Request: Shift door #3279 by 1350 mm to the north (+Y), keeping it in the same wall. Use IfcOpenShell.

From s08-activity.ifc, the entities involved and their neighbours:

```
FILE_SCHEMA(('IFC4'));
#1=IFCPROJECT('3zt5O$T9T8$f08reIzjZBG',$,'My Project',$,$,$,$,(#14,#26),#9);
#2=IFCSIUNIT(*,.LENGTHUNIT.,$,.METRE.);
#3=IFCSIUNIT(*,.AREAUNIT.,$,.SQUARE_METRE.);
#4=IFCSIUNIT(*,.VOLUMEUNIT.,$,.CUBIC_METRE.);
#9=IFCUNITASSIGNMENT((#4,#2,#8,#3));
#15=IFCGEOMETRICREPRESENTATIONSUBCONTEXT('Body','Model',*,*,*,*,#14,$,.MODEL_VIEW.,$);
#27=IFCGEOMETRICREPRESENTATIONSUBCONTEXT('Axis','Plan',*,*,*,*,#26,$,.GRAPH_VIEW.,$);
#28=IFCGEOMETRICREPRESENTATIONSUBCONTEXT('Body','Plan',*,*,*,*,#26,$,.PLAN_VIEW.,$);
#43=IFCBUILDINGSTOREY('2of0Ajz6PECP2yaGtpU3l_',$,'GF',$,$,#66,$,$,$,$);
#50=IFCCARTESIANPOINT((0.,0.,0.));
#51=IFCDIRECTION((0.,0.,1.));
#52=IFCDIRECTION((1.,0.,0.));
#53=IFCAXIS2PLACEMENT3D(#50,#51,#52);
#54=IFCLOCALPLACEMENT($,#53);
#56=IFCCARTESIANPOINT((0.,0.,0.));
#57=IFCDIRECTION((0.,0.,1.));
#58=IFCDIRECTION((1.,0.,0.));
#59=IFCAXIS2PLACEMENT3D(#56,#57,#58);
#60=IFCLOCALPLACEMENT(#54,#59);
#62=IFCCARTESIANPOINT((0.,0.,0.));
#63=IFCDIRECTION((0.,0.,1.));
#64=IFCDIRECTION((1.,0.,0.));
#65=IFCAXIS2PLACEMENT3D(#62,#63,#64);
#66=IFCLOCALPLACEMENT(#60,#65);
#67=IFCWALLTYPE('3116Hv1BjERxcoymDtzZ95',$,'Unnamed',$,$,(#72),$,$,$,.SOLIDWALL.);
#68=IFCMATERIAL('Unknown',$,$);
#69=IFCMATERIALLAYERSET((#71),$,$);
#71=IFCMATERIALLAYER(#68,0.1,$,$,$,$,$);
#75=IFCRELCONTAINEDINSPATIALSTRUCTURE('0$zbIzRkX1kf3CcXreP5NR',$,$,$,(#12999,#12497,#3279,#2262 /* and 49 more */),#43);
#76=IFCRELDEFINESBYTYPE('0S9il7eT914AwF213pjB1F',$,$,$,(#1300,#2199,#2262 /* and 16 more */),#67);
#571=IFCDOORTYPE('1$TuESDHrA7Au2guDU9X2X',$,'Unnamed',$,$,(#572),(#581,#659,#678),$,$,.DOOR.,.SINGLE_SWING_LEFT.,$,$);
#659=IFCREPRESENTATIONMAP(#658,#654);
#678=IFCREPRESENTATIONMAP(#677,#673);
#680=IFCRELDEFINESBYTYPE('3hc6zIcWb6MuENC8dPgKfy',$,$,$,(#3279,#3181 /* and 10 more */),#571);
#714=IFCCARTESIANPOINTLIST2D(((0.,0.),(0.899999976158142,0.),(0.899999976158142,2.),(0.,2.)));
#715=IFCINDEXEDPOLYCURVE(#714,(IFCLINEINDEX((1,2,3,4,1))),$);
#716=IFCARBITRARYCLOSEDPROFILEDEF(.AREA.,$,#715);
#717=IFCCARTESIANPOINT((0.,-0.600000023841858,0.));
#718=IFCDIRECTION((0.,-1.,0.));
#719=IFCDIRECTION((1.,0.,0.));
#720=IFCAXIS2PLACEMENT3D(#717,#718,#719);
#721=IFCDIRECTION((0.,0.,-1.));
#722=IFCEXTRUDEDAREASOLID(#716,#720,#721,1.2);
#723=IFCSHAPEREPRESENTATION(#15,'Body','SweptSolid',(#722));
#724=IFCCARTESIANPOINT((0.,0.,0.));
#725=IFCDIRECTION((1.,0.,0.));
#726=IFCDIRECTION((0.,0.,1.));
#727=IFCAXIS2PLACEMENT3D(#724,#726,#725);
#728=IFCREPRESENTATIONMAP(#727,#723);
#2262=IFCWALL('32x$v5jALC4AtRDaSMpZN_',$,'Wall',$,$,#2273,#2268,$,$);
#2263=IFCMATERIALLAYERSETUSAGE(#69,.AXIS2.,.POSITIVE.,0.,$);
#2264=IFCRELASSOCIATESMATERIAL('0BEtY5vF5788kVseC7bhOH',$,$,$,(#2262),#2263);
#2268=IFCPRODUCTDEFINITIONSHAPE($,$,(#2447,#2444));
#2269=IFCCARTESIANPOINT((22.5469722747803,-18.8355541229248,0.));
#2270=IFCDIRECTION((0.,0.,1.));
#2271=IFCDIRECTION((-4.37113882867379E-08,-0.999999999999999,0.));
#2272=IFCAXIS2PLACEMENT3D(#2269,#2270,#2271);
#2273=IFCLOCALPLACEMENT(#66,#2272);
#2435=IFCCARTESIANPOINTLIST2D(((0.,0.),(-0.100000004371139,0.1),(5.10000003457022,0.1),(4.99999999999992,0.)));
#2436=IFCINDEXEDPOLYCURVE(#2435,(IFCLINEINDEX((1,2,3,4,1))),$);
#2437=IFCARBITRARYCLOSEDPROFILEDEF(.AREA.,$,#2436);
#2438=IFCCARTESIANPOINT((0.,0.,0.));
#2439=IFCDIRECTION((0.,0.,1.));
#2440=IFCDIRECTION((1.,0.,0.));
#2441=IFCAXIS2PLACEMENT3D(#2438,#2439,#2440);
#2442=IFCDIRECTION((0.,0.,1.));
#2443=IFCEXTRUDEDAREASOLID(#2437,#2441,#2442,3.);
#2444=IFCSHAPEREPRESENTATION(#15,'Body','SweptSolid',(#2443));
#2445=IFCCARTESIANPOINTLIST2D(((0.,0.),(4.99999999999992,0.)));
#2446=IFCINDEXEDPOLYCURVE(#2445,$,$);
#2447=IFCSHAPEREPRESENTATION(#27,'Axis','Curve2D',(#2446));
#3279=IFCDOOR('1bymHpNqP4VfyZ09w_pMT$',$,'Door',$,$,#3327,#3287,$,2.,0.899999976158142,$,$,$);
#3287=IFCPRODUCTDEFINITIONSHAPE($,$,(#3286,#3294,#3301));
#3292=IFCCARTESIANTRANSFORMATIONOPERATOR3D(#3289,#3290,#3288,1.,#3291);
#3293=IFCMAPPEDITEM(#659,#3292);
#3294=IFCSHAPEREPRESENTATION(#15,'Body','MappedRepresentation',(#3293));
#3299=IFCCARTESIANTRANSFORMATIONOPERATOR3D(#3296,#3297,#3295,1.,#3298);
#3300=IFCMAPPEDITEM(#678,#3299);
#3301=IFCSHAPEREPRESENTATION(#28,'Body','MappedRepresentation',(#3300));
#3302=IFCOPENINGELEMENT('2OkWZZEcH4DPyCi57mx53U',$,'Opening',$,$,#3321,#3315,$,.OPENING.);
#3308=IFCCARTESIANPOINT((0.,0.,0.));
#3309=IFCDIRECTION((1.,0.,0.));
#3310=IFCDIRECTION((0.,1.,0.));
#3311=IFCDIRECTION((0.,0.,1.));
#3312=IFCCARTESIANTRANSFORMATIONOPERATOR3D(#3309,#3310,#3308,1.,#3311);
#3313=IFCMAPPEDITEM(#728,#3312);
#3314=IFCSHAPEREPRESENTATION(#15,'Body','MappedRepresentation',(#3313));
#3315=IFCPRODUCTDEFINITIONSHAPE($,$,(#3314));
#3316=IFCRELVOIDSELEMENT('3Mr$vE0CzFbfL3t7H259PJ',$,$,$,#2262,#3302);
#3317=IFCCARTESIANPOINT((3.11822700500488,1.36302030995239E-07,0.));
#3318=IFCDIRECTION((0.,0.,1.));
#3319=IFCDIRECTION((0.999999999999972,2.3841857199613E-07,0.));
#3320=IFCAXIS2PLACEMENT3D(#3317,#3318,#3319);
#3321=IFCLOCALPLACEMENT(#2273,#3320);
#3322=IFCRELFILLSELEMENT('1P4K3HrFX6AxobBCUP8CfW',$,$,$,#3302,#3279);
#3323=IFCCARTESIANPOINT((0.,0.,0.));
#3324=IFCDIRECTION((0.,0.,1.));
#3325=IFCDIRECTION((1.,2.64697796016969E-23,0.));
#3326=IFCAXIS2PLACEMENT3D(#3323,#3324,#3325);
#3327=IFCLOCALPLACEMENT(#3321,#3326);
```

```python
import ifcopenshell
import ifcopenshell.api.geometry
import ifcopenshell.util.placement

model = ifcopenshell.open("s08-activity.ifc")

door = model.by_guid("1bymHpNqP4VfyZ09w_pMT$")
opening = door.FillsVoids[0].RelatingOpeningElement
wall = opening.VoidsElements[0].RelatingBuildingElement

wall_matrix = ifcopenshell.util.placement.get_local_placement(wall.ObjectPlacement)
shift = wall_matrix[:3, 0] * -1.35
before = ifcopenshell.util.placement.get_local_placement(door.ObjectPlacement)[:3, 3].copy()

# The door is placed relative to its opening, so it follows when the opening moves.
matrix = ifcopenshell.util.placement.get_local_placement(opening.ObjectPlacement)
matrix[:3, 3] += shift
ifcopenshell.api.geometry.edit_object_placement(
    model, product=opening, matrix=matrix, is_si=False, should_transform_children=True
)

after = ifcopenshell.util.placement.get_local_placement(door.ObjectPlacement)[:3, 3]
print("door moved by", (after - before).round(3) + 0.0)

model.write("s08-activity_rev.ifc")
```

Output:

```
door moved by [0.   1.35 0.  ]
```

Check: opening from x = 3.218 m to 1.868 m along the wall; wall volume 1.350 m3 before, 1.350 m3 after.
